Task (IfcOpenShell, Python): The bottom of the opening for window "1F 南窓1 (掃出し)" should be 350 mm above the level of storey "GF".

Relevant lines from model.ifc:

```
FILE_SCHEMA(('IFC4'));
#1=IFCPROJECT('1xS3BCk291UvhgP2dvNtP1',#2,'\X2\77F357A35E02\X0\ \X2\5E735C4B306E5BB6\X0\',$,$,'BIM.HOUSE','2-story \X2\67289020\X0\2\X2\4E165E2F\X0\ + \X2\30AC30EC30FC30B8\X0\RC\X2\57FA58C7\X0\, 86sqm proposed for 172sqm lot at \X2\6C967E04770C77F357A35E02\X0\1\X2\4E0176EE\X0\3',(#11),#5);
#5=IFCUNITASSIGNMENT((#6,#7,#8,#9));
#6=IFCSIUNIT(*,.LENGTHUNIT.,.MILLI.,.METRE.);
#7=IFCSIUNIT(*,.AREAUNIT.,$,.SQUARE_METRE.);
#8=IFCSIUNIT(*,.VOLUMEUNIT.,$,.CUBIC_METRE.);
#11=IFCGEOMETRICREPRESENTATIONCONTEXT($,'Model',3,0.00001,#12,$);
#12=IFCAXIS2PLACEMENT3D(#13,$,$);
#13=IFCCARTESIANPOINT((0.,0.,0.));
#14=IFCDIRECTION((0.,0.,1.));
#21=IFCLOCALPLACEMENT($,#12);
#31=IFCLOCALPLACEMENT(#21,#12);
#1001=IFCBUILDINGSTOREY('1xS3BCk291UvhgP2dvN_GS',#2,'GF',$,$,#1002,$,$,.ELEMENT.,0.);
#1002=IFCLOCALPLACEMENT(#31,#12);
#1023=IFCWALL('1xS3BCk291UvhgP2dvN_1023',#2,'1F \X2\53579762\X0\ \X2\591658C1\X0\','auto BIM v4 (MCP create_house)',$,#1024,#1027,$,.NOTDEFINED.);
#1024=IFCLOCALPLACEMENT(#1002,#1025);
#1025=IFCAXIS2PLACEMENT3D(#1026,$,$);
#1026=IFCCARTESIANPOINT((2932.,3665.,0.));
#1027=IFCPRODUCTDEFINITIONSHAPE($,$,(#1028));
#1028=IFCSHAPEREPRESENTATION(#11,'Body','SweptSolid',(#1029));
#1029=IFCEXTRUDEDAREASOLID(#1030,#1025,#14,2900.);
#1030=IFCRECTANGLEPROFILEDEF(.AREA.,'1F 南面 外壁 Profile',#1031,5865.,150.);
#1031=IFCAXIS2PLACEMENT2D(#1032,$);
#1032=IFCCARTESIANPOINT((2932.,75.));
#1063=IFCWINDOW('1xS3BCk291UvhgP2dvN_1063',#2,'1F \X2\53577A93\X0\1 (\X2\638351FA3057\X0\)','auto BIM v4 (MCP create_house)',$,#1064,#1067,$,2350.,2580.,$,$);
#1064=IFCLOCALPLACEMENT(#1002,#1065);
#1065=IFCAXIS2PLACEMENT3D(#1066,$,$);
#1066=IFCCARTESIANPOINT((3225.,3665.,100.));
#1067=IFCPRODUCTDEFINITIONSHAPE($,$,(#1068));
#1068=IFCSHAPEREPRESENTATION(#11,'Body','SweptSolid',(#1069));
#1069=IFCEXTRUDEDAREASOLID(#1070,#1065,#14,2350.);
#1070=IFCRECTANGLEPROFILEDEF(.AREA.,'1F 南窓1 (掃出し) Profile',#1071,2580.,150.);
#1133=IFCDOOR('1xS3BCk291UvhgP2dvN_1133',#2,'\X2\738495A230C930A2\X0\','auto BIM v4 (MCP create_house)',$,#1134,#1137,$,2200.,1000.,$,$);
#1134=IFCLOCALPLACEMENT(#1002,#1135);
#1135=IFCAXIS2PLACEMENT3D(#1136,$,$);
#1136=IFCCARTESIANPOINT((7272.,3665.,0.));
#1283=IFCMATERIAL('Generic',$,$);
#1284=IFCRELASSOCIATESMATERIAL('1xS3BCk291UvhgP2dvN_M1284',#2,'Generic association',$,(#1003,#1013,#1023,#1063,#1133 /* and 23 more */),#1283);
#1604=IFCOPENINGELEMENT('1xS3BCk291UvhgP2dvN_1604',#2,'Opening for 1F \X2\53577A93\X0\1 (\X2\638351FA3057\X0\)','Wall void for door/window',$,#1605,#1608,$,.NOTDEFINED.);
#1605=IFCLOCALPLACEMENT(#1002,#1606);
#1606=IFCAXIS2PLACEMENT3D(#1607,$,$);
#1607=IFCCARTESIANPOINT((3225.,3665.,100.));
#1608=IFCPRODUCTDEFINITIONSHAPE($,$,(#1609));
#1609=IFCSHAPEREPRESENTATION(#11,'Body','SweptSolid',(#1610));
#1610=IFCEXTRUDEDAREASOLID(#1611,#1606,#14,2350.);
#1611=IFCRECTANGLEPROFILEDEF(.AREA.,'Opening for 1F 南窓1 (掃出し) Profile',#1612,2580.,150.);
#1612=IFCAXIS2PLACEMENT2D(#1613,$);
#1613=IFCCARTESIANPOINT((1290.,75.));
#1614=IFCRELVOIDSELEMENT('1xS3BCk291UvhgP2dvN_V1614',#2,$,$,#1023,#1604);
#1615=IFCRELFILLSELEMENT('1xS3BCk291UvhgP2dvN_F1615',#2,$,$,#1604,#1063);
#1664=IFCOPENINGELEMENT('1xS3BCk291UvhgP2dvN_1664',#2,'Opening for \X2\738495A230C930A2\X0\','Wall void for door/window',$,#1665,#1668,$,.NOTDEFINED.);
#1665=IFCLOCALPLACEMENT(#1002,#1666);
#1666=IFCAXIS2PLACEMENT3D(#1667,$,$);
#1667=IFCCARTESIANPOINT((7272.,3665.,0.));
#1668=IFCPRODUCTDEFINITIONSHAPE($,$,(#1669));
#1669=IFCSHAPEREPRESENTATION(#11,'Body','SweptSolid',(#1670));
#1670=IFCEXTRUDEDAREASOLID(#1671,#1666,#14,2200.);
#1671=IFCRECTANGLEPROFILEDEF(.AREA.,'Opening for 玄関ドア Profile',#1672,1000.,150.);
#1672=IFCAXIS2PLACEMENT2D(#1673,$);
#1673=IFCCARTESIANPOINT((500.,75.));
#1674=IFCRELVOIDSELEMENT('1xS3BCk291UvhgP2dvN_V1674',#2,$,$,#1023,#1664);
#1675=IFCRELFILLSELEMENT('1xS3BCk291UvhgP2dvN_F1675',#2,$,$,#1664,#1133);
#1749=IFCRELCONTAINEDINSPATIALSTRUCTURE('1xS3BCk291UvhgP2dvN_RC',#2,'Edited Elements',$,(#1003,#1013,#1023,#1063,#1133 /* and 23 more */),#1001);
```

```python
import numpy as np
import ifcopenshell
import ifcopenshell.api.geometry
import ifcopenshell.geom
import ifcopenshell.util.element
import ifcopenshell.util.placement
import ifcopenshell.util.shape
import ifcopenshell.util.unit

model = ifcopenshell.open("model.ifc")
unit_scale = ifcopenshell.util.unit.calculate_unit_scale(model)

window = model.by_guid("1xS3BCk291UvhgP2dvN_1063")
opening = window.FillsVoids[0].RelatingOpeningElement
storey = ifcopenshell.util.element.get_container(window, ifc_class="IfcBuildingStorey")
level = ifcopenshell.util.placement.get_local_placement(storey.ObjectPlacement)[2, 3]

# The opening's origin need not be at the sill, so measure its lowest point.
shape = ifcopenshell.geom.create_shape(ifcopenshell.geom.settings(), opening)
bottom = ifcopenshell.util.shape.get_shape_bottom_elevation(shape, shape.geometry) / unit_scale
dz = level + 0.35 / unit_scale - bottom

shift = np.array([0.0, 0.0, dz])
# The window is not placed relative to its opening, so move both.
for product in (opening, window):
    matrix = ifcopenshell.util.placement.get_local_placement(product.ObjectPlacement)
    matrix[:3, 3] += shift
    ifcopenshell.api.geometry.edit_object_placement(model, product=product, matrix=matrix, is_si=False)

print(f"moved by {dz * unit_scale:+.3f} m")

model.write("model_v2.ifc")
```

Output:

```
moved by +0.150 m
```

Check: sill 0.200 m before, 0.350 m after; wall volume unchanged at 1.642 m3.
